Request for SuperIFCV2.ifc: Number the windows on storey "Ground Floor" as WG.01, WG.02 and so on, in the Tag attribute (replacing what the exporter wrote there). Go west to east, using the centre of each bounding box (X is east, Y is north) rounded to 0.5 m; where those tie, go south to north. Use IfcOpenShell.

First a look at what the model holds.

```python
import ifcopenshell
import ifcopenshell.util.element
import ifcopenshell.util.placement

model = ifcopenshell.open("SuperIFCV2.ifc")
print(model.schema)
storey = next(s for s in model.by_type("IfcBuildingStorey") if s.Name == "Ground Floor")
windows = [e for e in ifcopenshell.util.element.get_decomposition(storey) if e.is_a("IfcWindow")]
for e in sorted(windows, key=lambda e: e.id()):
    origin = ifcopenshell.util.placement.get_local_placement(e.ObjectPlacement)[:3, 3]
    print(e.id(), e.Tag, e.Name, origin.round(2) + 0.0, sep=" | ")
```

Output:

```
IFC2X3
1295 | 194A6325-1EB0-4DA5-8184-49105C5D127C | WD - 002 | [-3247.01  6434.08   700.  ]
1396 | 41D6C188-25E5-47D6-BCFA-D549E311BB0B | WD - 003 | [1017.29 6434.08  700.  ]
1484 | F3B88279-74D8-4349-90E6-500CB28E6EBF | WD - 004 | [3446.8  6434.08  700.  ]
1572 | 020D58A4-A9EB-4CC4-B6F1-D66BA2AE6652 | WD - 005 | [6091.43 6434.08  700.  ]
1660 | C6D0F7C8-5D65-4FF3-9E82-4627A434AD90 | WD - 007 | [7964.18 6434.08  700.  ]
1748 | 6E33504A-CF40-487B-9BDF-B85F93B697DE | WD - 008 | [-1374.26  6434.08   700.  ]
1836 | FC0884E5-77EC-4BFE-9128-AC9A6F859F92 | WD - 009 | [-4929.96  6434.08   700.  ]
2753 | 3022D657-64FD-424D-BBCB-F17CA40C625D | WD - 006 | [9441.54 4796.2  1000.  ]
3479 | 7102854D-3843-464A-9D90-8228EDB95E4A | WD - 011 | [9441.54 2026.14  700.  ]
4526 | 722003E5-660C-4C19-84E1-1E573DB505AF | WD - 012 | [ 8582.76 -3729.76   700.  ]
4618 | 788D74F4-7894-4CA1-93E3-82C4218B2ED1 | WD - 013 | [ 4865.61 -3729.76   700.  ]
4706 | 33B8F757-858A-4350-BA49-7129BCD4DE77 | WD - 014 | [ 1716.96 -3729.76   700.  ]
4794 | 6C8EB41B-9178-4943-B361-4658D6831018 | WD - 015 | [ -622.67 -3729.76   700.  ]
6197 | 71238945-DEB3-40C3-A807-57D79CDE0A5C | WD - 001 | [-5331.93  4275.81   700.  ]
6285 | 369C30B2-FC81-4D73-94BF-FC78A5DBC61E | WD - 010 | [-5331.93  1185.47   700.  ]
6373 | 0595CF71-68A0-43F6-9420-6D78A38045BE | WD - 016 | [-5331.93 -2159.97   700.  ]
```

```python
import ifcopenshell
import ifcopenshell.geom
import ifcopenshell.util.element
import ifcopenshell.util.shape

model = ifcopenshell.open("SuperIFCV2.ifc")
settings = ifcopenshell.geom.settings()
settings.set("use-world-coords", True)


def centre(element):
    shape = ifcopenshell.geom.create_shape(settings, element)
    return ifcopenshell.util.shape.get_bbox_centroid(shape.geometry)


storey = next(s for s in model.by_type("IfcBuildingStorey") if s.Name == "Ground Floor")
windows = [e for e in ifcopenshell.util.element.get_decomposition(storey) if e.is_a("IfcWindow")]

# Insertion points can sit at a corner or the storey origin, so sort by the geometry (in metres).
centres = {e: centre(e) for e in windows}
windows.sort(key=lambda e: (round(centres[e][0] / 0.5), centres[e][1]))

for i, e in enumerate(windows, start=1):
    number = f"WG.{i:02d}"
    e.Tag = number
    print(e.id(), number)

model.write("SuperIFCV2_edited.ifc")
```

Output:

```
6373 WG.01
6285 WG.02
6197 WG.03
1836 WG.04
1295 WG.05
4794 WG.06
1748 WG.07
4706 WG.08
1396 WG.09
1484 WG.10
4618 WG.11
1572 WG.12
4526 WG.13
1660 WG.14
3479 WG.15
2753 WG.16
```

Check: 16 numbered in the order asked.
